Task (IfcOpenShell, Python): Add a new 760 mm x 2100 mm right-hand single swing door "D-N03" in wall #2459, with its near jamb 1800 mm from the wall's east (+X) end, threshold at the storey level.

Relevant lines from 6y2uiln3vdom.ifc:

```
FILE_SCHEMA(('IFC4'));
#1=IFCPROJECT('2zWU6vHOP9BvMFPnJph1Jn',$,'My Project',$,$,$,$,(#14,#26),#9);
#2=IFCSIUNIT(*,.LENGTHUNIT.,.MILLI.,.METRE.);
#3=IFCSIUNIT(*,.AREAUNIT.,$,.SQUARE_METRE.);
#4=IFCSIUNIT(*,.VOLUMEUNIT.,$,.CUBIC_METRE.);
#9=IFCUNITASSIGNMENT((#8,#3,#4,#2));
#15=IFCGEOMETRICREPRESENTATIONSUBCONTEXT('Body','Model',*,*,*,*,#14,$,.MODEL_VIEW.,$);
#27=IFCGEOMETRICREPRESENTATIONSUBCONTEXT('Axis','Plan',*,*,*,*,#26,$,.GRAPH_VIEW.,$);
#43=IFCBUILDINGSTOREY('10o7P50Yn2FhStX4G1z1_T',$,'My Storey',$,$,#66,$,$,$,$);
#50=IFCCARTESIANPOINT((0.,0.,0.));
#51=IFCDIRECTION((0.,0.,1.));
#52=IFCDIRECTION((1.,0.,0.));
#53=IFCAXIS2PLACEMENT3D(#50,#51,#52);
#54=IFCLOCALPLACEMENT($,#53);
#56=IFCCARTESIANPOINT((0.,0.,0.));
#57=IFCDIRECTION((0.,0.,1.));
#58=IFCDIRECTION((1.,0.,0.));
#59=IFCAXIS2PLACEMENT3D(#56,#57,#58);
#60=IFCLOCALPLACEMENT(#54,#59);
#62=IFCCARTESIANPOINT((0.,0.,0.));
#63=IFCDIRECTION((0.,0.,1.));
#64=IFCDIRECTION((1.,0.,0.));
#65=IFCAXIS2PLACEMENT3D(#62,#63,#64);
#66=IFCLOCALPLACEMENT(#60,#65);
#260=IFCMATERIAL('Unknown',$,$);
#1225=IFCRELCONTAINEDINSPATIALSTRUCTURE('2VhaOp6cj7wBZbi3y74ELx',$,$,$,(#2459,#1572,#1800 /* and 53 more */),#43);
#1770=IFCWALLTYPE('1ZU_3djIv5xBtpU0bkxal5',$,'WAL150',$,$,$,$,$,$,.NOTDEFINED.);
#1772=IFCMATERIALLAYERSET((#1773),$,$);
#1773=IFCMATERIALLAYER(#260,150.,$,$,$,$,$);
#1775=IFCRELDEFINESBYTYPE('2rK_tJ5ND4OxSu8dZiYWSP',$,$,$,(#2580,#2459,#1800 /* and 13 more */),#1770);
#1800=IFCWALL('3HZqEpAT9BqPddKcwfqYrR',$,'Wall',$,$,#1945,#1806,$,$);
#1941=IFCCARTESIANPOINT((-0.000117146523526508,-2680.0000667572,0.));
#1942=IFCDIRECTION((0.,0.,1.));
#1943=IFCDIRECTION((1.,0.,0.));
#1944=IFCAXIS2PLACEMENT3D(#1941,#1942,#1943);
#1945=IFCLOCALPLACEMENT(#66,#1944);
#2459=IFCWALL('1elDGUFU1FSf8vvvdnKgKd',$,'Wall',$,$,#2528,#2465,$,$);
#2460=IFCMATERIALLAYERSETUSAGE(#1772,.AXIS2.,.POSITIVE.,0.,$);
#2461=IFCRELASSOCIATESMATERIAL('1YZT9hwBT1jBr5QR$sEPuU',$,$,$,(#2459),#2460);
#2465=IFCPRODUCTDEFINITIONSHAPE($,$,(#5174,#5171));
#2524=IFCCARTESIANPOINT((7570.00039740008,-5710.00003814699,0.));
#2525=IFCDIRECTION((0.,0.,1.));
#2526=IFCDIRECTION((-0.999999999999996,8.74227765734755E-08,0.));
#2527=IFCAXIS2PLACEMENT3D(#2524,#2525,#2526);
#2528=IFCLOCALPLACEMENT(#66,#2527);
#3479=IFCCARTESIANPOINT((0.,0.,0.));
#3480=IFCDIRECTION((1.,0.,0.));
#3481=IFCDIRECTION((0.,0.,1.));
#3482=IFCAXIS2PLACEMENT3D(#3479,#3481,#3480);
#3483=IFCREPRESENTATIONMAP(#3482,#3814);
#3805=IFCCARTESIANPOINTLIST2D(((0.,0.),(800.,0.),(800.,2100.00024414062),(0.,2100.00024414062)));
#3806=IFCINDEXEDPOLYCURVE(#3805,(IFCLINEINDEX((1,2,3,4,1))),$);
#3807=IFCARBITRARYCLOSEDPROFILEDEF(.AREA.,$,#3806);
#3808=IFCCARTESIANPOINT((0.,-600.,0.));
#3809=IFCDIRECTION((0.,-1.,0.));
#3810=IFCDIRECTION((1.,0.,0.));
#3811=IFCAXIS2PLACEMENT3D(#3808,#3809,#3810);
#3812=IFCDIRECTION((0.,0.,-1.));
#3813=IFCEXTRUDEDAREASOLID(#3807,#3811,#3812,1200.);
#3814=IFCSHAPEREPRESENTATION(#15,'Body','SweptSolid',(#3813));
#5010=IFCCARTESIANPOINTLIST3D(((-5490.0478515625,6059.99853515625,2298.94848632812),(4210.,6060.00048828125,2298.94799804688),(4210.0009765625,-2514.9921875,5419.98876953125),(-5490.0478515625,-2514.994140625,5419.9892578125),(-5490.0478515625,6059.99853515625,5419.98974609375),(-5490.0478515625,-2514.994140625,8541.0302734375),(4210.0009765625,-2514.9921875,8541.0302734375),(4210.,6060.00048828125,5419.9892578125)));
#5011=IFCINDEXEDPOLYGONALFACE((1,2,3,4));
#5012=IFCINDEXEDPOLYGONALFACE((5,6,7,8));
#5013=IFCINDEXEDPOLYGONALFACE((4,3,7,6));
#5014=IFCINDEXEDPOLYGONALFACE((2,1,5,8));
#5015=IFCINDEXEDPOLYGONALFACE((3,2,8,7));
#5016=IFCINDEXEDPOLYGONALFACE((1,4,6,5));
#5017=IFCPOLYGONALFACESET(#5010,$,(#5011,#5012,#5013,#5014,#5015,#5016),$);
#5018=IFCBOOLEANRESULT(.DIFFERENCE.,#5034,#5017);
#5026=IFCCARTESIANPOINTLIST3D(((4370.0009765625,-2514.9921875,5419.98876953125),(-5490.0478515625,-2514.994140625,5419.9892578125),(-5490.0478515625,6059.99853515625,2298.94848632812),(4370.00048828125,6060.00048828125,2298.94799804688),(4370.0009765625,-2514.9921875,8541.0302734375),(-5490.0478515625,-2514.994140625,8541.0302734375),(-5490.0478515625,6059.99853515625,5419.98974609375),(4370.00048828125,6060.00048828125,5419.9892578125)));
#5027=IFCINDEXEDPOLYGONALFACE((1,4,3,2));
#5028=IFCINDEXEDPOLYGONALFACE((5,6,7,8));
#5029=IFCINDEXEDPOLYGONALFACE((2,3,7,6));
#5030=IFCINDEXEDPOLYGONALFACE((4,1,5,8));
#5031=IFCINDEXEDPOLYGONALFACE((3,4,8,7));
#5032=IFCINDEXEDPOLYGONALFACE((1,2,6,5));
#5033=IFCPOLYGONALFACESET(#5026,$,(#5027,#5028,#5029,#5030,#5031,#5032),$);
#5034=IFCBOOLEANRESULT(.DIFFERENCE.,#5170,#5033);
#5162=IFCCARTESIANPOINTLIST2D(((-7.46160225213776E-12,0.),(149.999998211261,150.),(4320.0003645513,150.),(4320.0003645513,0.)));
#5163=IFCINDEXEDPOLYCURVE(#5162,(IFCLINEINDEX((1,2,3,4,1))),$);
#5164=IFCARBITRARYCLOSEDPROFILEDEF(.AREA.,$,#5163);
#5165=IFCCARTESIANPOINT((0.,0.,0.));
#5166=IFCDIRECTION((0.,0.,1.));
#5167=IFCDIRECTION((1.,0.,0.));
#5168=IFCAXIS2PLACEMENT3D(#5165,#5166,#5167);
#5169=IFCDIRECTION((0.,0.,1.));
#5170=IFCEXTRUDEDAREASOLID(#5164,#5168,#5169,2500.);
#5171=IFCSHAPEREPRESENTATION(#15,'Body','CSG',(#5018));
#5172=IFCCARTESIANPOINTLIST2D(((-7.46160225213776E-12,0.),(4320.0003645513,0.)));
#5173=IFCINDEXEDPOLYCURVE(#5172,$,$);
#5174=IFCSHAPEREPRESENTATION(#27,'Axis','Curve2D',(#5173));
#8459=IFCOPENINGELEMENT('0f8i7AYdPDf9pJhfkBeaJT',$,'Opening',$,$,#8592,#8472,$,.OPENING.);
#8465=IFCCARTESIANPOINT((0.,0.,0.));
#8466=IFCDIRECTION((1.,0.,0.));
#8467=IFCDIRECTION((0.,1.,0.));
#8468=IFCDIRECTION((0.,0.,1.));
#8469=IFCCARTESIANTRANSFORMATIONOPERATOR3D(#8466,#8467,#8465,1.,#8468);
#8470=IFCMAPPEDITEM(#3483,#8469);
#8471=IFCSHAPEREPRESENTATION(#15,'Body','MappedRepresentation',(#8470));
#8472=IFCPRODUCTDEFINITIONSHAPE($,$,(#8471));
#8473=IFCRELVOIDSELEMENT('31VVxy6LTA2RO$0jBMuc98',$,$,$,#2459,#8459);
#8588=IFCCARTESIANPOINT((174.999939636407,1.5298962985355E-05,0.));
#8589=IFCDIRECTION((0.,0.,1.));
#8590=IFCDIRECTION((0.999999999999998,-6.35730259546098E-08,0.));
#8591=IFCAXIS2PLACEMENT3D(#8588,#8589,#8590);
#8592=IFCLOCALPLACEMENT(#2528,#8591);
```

```python
import numpy as np
import ifcopenshell
import ifcopenshell.api.feature
import ifcopenshell.api.geometry
import ifcopenshell.api.root
import ifcopenshell.api.spatial
import ifcopenshell.geom
import ifcopenshell.util.element
import ifcopenshell.util.placement
import ifcopenshell.util.representation
import ifcopenshell.util.shape
import ifcopenshell.util.unit

model = ifcopenshell.open("6y2uiln3vdom.ifc")
unit_scale = ifcopenshell.util.unit.calculate_unit_scale(model)
settings = ifcopenshell.geom.settings()


def volume(element):
    """Net volume in cubic metres, openings subtracted."""
    shape = ifcopenshell.geom.create_shape(settings, element)
    return ifcopenshell.util.shape.get_volume(shape.geometry)


wall = model.by_id(2459)
storey = ifcopenshell.util.element.get_container(wall, ifc_class="IfcBuildingStorey")
context = ifcopenshell.util.representation.get_context(model, "Model", "Body", "MODEL_VIEW")
before = volume(wall)

width, height, from_end, sill = 0.76, 2.1, 1.8, 0.0  # metres

# The wall runs along its own X axis, and the end named is its -X end.
wall_shape = ifcopenshell.geom.create_shape(settings, wall)
x, y, z = ifcopenshell.util.shape.get_vertices(wall_shape.geometry).T
start = x.min() + from_end
face, thickness = float(y.min()), float(y.max() - y.min())
wall_matrix = ifcopenshell.util.placement.get_local_placement(wall.ObjectPlacement)
level = ifcopenshell.util.placement.get_local_placement(storey.ObjectPlacement)[2, 3]


def in_wall(x, y):
    """Placement at x, y metres in the wall's axes, at sill height."""
    matrix = wall_matrix.copy()
    matrix[:, 3] = wall_matrix @ np.array([x / unit_scale, y / unit_scale, 0.0, 1.0])
    matrix[2, 3] = level + sill / unit_scale
    return matrix


# Opening: a box that overshoots both wall faces by 50 mm.
opening = ifcopenshell.api.root.create_entity(model, ifc_class="IfcOpeningElement", predefined_type="OPENING")
box = ifcopenshell.api.geometry.add_wall_representation(
    model, context=context, length=width, height=height, thickness=thickness + 0.1
)
ifcopenshell.api.geometry.assign_representation(model, product=opening, representation=box)
ifcopenshell.api.geometry.edit_object_placement(model, product=opening, matrix=in_wall(start, face - 0.05), is_si=False)
ifcopenshell.api.feature.add_feature(model, feature=opening, element=wall)

door = ifcopenshell.api.root.create_entity(model, ifc_class="IfcDoor", name="D-N03", predefined_type="DOOR")
door.OverallWidth, door.OverallHeight = width / unit_scale, height / unit_scale
door.OperationType = "SINGLE_SWING_RIGHT"
body = ifcopenshell.api.geometry.add_door_representation(
    model,
    context=context,
    overall_width=door.OverallWidth,
    overall_height=door.OverallHeight,
    operation_type="SINGLE_SWING_RIGHT",
    lining_properties={"LiningDepth": thickness / unit_scale, "ThresholdDepth": thickness / unit_scale},
)
ifcopenshell.api.geometry.assign_representation(model, product=door, representation=body)
ifcopenshell.api.spatial.assign_container(model, products=[door], relating_structure=storey)
ifcopenshell.api.feature.add_filling(model, opening=opening, element=door)

# The lining spans the wall, so the door starts at the wall face.
ifcopenshell.api.geometry.edit_object_placement(model, product=door, matrix=in_wall(start, face), is_si=False)

after = volume(wall)

print(f"wall volume {before:.3f} -> {after:.3f} m3")

model.write("6y2uiln3vdom-out.ifc")
```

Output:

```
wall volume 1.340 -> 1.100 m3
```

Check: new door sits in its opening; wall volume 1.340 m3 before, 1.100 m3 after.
